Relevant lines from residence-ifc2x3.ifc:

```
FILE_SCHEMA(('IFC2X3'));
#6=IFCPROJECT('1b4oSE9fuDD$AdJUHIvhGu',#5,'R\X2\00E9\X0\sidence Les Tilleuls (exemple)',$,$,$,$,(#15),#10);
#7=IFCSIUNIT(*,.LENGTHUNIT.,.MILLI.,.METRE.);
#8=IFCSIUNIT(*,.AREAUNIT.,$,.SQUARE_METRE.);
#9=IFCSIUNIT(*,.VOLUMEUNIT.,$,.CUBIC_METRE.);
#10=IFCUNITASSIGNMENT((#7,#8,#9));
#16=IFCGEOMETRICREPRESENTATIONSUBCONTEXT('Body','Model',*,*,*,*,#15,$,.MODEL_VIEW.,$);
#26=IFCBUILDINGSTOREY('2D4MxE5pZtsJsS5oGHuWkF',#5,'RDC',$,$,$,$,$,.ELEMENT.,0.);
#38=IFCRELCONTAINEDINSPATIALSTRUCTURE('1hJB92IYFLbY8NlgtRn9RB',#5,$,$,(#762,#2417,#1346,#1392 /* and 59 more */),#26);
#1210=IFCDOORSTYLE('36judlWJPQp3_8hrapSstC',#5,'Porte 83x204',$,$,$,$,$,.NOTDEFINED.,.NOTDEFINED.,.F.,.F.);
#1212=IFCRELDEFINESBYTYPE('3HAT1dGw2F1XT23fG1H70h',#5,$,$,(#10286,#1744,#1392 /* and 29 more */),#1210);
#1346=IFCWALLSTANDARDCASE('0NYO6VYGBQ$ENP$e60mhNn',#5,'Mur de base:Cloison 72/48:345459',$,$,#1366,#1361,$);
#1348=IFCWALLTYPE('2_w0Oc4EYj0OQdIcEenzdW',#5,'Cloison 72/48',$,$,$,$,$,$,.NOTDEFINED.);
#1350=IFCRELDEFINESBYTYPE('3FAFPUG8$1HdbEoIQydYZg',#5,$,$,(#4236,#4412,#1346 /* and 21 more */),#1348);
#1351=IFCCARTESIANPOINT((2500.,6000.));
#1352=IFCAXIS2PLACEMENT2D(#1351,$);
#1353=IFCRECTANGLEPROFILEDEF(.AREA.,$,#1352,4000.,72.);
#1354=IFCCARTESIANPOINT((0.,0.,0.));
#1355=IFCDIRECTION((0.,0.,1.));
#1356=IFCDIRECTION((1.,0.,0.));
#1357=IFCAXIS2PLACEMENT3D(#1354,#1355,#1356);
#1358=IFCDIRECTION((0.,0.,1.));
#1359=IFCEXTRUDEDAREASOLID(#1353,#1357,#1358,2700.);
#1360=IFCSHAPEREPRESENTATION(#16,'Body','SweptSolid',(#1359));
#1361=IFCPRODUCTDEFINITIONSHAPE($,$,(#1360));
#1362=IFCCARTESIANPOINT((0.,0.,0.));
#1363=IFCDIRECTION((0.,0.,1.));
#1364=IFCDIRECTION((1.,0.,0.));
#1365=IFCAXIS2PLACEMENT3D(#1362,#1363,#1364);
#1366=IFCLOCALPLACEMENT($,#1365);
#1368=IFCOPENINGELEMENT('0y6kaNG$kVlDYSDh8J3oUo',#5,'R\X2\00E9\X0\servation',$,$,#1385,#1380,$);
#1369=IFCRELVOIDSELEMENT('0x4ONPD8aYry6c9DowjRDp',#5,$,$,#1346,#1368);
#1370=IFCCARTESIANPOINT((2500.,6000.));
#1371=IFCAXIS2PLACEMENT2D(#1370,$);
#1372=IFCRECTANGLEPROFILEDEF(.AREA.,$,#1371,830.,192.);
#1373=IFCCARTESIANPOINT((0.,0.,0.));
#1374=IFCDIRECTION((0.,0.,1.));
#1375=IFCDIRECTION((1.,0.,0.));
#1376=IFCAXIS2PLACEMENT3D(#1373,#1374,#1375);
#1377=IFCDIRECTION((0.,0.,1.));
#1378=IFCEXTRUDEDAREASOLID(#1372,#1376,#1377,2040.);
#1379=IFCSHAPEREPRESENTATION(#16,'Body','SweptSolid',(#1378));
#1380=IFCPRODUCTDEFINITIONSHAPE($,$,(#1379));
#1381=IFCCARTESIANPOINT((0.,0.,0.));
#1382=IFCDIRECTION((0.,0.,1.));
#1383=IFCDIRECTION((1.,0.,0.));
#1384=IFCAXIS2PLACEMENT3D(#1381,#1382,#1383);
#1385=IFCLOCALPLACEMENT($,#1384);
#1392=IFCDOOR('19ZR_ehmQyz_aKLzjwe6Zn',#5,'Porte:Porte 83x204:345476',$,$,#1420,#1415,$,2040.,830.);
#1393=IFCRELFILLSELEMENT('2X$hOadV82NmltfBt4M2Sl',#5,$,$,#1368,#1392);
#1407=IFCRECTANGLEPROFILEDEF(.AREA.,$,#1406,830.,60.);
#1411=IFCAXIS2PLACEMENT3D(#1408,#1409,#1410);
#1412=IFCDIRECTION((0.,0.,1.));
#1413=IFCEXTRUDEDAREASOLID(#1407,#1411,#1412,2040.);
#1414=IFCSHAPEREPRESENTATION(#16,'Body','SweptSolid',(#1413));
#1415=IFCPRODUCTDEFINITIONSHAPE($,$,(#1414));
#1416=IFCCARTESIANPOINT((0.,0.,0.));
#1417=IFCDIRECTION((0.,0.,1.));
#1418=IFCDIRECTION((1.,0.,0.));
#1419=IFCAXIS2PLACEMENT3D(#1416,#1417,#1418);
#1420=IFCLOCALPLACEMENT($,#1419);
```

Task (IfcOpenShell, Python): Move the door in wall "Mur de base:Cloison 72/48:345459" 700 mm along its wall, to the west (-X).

```python
import ifcopenshell
import ifcopenshell.api.geometry
import ifcopenshell.util.placement

model = ifcopenshell.open("residence-ifc2x3.ifc")

door = model.by_guid("19ZR_ehmQyz_aKLzjwe6Zn")
opening = door.FillsVoids[0].RelatingOpeningElement
wall = opening.VoidsElements[0].RelatingBuildingElement

wall_matrix = ifcopenshell.util.placement.get_local_placement(wall.ObjectPlacement)
shift = wall_matrix[:3, 0] * -700.0
before = ifcopenshell.util.placement.get_local_placement(door.ObjectPlacement)[:3, 3].copy()

# The door is not placed relative to its opening, so move both.
for product in (opening, door):
    matrix = ifcopenshell.util.placement.get_local_placement(product.ObjectPlacement)
    matrix[:3, 3] += shift
    ifcopenshell.api.geometry.edit_object_placement(model, product=product, matrix=matrix, is_si=False)

after = ifcopenshell.util.placement.get_local_placement(door.ObjectPlacement)[:3, 3]
print("door moved by", (after - before).round(3) + 0.0)

model.write("residence-ifc2x3_v2.ifc")
```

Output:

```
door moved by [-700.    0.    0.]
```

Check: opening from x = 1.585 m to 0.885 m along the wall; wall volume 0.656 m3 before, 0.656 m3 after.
